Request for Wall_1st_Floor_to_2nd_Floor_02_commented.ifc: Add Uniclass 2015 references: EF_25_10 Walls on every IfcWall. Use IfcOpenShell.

First a look at what the model holds.

```python
import ifcopenshell

model = ifcopenshell.open("Wall_1st_Floor_to_2nd_Floor_02_commented.ifc")
print(model.schema)
print("classifications:", [c.Name for c in model.by_type("IfcClassification")])
for ifc_class in ("IfcDoor", "IfcRoof", "IfcStair", "IfcWall", "IfcWindow"):
    print(ifc_class, len(model.by_type(ifc_class)))
```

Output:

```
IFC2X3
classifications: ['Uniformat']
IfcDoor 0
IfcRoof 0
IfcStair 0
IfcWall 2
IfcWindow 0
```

```python
import ifcopenshell
import ifcopenshell.api.classification

model = ifcopenshell.open("Wall_1st_Floor_to_2nd_Floor_02_commented.ifc")

# IFC2X3 requires Source and Edition and has no link from the project to the system.
system = model.create_entity("IfcClassification", Source="NBS", Edition="2015", Name="Uniclass 2015")

codes = {
    "IfcWall": ("EF_25_10", "Walls"),
}
for ifc_class, (code, name) in codes.items():
    products = model.by_type(ifc_class)
    ifcopenshell.api.classification.add_reference(
        model, products=products, classification=system, identification=code, name=name
    )
    print(code, len(products))

model.write("Wall_1st_Floor_to_2nd_Floor_02_commented_v2.ifc")
```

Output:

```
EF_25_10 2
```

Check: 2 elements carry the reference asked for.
